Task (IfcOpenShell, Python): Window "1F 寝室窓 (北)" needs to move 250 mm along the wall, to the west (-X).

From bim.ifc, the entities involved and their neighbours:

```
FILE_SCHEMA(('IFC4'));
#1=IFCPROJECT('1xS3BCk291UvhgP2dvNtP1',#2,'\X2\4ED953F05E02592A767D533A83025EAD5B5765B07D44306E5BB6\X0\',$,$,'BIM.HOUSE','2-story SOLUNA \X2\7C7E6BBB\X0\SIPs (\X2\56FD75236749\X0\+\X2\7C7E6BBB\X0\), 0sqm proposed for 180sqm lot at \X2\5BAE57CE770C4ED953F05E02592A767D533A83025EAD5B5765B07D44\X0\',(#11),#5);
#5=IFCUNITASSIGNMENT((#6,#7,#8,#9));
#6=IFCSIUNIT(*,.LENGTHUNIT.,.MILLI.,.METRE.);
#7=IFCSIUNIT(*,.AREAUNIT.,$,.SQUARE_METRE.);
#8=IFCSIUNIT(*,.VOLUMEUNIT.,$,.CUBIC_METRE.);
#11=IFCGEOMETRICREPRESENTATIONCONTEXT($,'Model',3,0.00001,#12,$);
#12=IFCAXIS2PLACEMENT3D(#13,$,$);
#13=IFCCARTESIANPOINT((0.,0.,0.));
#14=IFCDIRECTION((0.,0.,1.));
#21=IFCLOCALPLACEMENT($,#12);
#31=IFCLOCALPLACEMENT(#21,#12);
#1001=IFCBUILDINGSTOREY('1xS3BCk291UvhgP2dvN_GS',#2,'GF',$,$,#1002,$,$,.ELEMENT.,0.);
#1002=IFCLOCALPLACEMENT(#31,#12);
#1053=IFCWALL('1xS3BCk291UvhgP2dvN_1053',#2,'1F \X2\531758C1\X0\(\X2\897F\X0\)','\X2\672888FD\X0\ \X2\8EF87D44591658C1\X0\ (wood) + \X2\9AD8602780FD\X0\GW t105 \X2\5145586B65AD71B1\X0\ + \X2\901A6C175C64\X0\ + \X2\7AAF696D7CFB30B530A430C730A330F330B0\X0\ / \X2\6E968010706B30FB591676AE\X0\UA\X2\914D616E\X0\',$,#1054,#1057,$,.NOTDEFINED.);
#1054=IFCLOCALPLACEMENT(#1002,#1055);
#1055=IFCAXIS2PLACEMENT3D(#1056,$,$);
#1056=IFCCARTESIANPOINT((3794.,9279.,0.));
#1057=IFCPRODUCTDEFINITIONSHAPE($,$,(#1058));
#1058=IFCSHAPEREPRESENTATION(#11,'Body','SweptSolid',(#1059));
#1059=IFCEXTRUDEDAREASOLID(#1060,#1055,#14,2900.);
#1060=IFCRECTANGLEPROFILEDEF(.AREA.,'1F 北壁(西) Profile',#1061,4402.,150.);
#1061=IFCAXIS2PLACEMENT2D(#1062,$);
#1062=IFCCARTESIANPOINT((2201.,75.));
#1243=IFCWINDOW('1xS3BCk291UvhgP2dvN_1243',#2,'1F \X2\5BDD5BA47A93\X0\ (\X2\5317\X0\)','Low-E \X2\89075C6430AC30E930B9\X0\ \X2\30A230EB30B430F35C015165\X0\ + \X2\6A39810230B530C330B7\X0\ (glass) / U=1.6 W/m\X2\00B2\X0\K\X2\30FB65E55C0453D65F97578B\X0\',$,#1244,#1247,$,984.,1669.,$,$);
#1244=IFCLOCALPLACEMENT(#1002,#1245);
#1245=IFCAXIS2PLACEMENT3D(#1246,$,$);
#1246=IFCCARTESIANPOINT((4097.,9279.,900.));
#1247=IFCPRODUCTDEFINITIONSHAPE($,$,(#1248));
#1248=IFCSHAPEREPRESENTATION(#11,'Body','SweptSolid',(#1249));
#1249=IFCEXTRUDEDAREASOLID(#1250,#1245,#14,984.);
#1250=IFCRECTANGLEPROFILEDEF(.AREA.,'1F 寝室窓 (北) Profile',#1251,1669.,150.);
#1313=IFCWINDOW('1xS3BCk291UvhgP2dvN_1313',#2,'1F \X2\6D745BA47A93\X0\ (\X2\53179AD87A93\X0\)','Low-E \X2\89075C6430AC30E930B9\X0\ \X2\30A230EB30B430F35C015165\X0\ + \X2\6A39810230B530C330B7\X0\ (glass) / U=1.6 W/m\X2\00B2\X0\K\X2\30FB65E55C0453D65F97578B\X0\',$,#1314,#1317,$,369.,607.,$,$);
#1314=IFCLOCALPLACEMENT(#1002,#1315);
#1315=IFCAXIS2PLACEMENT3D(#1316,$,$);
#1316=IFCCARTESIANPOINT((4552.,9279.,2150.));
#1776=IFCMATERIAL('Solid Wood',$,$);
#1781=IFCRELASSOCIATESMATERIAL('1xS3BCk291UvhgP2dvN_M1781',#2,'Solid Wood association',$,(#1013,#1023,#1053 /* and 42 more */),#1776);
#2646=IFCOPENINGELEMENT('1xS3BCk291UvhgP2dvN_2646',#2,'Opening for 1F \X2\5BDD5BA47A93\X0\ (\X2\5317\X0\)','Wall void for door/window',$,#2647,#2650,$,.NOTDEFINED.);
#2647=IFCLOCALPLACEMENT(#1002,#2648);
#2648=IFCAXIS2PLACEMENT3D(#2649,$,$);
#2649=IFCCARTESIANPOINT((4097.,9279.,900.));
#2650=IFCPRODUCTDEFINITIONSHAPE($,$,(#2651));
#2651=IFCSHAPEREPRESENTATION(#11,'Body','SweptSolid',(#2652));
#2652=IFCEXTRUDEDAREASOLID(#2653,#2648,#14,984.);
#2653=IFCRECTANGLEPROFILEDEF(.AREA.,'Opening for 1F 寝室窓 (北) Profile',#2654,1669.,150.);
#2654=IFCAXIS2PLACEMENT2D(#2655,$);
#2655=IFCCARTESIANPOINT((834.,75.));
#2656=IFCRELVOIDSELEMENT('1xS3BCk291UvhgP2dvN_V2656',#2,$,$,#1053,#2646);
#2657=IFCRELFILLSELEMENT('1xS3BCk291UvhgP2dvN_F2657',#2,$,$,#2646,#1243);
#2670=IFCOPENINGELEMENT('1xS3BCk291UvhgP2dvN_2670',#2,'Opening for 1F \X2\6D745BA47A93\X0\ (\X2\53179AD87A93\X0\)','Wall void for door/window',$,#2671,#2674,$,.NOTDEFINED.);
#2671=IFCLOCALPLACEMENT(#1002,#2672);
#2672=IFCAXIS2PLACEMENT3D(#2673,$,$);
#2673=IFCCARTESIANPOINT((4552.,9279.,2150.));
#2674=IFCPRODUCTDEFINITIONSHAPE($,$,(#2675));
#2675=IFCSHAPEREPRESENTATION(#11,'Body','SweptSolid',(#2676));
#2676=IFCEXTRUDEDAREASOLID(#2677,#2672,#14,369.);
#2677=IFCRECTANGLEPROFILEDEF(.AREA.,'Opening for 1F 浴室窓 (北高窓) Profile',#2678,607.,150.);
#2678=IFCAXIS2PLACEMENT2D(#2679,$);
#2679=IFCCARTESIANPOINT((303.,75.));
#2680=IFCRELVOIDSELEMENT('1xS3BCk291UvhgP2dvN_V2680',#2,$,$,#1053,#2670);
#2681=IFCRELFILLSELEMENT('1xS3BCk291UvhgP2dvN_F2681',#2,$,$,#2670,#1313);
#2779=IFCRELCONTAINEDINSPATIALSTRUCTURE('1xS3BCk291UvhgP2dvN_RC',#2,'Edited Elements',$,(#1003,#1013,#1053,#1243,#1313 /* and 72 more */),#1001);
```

```python
import ifcopenshell
import ifcopenshell.api.geometry
import ifcopenshell.util.placement
import ifcopenshell.util.unit

model = ifcopenshell.open("bim.ifc")
unit_scale = ifcopenshell.util.unit.calculate_unit_scale(model)

window = model.by_guid("1xS3BCk291UvhgP2dvN_1243")
opening = window.FillsVoids[0].RelatingOpeningElement
wall = opening.VoidsElements[0].RelatingBuildingElement

wall_matrix = ifcopenshell.util.placement.get_local_placement(wall.ObjectPlacement)
shift = wall_matrix[:3, 0] * -0.25 / unit_scale
before = ifcopenshell.util.placement.get_local_placement(window.ObjectPlacement)[:3, 3].copy()

# The window is not placed relative to its opening, so move both.
for product in (opening, window):
    matrix = ifcopenshell.util.placement.get_local_placement(product.ObjectPlacement)
    matrix[:3, 3] += shift
    ifcopenshell.api.geometry.edit_object_placement(model, product=product, matrix=matrix, is_si=False)

after = ifcopenshell.util.placement.get_local_placement(window.ObjectPlacement)[:3, 3]
print("window moved by", (after - before).round(3) + 0.0)

model.write("bim_v2.ifc")
```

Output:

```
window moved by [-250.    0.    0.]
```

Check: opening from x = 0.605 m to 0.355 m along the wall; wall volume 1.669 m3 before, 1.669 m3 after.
